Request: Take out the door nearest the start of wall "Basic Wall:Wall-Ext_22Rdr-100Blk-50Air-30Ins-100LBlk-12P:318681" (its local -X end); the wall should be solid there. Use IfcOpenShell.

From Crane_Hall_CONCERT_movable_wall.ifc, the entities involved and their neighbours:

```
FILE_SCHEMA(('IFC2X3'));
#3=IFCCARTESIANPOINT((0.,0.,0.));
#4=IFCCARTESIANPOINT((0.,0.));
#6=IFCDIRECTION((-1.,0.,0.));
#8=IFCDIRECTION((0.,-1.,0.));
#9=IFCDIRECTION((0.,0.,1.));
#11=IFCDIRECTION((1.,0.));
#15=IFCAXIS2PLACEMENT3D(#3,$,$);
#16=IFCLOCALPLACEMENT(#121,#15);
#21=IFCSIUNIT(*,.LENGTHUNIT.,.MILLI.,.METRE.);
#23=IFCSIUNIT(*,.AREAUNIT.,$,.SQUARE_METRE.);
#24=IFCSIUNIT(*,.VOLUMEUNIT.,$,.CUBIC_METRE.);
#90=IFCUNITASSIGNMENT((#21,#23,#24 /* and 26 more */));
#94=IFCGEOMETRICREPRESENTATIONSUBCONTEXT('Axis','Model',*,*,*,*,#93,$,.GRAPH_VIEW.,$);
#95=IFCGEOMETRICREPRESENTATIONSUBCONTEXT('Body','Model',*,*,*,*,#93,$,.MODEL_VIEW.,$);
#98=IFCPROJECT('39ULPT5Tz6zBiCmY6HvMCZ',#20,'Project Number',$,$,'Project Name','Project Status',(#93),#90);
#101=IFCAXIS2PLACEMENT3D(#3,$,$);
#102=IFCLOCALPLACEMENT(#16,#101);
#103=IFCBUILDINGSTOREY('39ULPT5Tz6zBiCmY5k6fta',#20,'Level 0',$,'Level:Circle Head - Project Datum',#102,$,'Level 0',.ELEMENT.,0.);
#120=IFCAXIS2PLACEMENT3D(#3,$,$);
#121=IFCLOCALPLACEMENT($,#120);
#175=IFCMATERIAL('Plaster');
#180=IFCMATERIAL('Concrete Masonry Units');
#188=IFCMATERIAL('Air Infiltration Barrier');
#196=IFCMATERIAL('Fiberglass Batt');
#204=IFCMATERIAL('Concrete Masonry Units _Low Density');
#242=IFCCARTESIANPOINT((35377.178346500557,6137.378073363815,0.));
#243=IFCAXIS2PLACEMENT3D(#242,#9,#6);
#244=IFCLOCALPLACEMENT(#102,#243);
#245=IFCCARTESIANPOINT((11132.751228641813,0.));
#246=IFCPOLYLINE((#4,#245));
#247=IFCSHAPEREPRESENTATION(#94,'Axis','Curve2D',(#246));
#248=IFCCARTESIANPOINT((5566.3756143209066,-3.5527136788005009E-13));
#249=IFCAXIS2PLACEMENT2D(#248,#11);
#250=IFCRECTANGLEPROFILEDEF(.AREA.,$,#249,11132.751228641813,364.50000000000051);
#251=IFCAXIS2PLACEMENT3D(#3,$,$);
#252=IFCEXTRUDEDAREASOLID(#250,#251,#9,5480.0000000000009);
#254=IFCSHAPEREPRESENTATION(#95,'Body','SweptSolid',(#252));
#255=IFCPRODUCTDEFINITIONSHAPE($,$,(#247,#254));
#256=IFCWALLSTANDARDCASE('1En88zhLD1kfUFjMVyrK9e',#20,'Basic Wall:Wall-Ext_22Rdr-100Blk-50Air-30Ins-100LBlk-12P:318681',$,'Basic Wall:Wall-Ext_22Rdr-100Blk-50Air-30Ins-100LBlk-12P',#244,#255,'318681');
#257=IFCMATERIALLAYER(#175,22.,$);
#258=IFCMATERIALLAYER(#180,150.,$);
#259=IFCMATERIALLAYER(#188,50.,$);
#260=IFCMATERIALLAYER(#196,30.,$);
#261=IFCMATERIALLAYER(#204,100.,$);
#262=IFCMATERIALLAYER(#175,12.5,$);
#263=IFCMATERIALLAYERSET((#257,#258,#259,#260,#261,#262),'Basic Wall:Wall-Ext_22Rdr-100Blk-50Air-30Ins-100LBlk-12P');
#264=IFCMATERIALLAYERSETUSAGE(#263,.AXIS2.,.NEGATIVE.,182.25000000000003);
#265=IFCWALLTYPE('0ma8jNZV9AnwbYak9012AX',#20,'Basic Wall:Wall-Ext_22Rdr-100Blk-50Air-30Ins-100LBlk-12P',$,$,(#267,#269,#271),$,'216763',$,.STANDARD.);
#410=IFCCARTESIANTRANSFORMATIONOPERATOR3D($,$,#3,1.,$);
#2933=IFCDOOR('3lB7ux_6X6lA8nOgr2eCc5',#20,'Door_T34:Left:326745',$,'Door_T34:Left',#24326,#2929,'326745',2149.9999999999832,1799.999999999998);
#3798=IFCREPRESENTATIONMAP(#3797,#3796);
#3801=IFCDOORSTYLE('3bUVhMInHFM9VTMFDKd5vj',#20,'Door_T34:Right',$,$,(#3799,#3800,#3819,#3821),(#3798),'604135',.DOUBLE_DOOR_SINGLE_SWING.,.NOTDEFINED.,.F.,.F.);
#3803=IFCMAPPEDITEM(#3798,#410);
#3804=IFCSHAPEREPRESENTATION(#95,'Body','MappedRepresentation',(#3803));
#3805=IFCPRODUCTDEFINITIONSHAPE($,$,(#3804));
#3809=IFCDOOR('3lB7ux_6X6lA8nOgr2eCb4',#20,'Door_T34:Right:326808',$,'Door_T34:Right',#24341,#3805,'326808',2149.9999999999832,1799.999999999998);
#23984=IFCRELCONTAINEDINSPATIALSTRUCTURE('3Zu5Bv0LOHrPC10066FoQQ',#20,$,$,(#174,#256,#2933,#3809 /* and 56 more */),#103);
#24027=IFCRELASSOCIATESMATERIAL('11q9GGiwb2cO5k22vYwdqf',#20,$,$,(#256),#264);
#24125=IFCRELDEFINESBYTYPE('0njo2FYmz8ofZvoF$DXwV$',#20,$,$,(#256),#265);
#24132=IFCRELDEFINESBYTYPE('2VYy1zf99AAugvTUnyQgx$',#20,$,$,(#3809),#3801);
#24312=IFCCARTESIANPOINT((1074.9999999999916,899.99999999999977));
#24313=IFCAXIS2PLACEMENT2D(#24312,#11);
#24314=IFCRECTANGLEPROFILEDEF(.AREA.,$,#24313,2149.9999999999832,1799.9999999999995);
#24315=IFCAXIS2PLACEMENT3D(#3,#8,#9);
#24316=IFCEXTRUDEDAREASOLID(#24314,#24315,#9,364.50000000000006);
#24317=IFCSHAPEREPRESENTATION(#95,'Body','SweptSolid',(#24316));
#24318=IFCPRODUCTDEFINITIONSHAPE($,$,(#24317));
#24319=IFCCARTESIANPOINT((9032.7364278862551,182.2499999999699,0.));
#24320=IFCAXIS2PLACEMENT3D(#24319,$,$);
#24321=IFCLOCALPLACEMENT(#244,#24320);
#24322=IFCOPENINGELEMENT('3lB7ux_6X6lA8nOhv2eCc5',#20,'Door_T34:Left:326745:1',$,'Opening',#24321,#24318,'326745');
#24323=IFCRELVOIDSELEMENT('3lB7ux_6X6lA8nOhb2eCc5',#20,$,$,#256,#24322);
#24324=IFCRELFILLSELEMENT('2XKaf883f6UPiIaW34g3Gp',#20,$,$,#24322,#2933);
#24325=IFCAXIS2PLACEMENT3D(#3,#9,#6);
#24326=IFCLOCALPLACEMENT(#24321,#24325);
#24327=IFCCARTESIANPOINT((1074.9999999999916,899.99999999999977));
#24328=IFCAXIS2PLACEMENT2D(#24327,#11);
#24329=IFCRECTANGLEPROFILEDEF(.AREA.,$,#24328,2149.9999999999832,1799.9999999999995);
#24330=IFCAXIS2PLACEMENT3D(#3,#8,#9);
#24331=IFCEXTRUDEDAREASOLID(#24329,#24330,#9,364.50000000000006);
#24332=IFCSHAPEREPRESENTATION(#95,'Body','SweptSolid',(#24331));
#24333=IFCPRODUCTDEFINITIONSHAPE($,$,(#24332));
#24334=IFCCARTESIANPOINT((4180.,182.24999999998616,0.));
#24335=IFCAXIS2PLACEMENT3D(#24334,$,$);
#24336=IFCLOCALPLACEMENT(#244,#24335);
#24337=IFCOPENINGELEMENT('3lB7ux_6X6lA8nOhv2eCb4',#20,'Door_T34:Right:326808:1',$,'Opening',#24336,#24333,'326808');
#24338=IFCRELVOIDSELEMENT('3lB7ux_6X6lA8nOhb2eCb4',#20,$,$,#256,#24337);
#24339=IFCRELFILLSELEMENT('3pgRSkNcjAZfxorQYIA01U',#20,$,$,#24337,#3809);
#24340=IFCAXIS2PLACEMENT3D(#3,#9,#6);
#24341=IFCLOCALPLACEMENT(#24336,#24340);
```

```python
import ifcopenshell
import ifcopenshell.api.feature
import ifcopenshell.api.root
import ifcopenshell.geom
import ifcopenshell.util.shape

model = ifcopenshell.open("Crane_Hall_CONCERT_movable_wall.ifc")
settings = ifcopenshell.geom.settings()


def volume(element):
    """Net volume in cubic metres, openings subtracted."""
    shape = ifcopenshell.geom.create_shape(settings, element)
    return ifcopenshell.util.shape.get_volume(shape.geometry)


door = model.by_guid("3lB7ux_6X6lA8nOgr2eCb4")
opening = door.FillsVoids[0].RelatingOpeningElement
wall = opening.VoidsElements[0].RelatingBuildingElement
before = volume(wall)

ifcopenshell.api.root.remove_product(model, product=door)
ifcopenshell.api.feature.remove_feature(model, feature=opening)

after = volume(wall)

print(f"wall volume {before:.3f} -> {after:.3f} m3")

model.write("Crane_Hall_CONCERT_movable_wall-out.ifc")
```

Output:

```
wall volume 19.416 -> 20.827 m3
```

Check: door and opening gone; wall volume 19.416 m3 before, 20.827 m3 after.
